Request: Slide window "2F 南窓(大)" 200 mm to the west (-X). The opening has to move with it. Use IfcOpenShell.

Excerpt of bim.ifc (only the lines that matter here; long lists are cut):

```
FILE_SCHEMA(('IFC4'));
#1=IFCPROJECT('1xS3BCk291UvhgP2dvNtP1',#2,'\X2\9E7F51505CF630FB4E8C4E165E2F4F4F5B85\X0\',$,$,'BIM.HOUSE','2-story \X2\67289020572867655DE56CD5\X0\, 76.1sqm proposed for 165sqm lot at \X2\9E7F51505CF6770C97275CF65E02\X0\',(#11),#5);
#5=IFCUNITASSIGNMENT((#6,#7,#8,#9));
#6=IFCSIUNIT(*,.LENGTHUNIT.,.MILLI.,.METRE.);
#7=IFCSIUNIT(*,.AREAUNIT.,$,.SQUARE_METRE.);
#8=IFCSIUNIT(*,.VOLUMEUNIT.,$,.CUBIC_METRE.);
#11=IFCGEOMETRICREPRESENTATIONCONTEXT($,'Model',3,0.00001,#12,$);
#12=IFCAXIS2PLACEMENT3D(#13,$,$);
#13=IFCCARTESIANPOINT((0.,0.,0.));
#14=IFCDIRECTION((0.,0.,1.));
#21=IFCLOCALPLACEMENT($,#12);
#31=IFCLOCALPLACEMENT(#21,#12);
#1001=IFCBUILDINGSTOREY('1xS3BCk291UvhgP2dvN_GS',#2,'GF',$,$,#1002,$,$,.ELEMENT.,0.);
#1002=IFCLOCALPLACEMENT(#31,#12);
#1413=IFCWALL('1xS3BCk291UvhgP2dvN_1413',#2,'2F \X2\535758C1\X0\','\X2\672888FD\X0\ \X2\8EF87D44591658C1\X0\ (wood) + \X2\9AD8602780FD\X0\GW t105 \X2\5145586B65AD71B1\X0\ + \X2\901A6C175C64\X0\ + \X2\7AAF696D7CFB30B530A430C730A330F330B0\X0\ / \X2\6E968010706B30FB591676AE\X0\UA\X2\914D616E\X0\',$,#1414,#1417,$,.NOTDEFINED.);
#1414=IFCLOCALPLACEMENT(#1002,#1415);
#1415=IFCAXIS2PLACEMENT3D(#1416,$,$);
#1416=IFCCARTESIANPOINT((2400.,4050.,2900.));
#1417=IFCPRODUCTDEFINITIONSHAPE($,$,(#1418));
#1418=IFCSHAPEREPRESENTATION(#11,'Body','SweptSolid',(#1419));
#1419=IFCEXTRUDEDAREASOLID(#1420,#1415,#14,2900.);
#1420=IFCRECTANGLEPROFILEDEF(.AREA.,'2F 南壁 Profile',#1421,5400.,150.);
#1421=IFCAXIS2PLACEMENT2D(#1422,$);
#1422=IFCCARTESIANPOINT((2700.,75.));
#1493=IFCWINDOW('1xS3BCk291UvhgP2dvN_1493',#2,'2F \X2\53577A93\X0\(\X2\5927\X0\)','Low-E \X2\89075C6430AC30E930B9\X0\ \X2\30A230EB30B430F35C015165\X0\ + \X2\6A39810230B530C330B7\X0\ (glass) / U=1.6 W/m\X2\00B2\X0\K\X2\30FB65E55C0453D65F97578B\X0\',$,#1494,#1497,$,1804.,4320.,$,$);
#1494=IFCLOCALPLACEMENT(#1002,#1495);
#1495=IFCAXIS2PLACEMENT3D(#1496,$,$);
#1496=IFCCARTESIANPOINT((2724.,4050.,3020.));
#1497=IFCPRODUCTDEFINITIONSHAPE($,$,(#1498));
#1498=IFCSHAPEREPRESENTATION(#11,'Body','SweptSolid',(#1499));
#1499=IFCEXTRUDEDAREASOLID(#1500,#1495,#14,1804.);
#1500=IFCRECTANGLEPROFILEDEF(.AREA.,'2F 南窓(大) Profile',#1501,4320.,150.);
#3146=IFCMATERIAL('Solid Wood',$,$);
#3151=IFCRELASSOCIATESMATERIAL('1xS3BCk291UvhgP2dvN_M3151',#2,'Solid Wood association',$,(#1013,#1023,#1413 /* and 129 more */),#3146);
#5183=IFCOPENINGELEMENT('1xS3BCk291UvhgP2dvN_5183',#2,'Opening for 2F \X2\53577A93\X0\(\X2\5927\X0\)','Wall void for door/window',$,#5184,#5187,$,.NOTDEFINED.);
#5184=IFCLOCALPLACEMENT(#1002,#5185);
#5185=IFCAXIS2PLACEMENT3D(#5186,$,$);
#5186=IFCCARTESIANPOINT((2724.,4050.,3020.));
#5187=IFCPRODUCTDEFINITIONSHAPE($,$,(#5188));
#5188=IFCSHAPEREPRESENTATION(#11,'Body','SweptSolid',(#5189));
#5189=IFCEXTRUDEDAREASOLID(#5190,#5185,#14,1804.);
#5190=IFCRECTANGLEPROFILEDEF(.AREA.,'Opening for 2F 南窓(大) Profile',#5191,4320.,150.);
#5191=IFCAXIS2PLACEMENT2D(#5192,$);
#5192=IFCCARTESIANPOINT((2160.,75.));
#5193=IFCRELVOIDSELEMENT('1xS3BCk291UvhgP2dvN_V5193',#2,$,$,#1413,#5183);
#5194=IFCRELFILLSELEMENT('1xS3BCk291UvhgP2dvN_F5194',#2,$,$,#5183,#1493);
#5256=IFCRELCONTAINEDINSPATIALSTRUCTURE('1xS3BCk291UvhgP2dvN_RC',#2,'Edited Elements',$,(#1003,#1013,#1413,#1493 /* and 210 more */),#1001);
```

```python
import ifcopenshell
import ifcopenshell.api.geometry
import ifcopenshell.util.placement
import ifcopenshell.util.unit

model = ifcopenshell.open("bim.ifc")
unit_scale = ifcopenshell.util.unit.calculate_unit_scale(model)

window = model.by_guid("1xS3BCk291UvhgP2dvN_1493")
opening = window.FillsVoids[0].RelatingOpeningElement
wall = opening.VoidsElements[0].RelatingBuildingElement

wall_matrix = ifcopenshell.util.placement.get_local_placement(wall.ObjectPlacement)
shift = wall_matrix[:3, 0] * -0.2 / unit_scale
before = ifcopenshell.util.placement.get_local_placement(window.ObjectPlacement)[:3, 3].copy()

# The window is not placed relative to its opening, so move both.
for product in (opening, window):
    matrix = ifcopenshell.util.placement.get_local_placement(product.ObjectPlacement)
    matrix[:3, 3] += shift
    ifcopenshell.api.geometry.edit_object_placement(model, product=product, matrix=matrix, is_si=False)

after = ifcopenshell.util.placement.get_local_placement(window.ObjectPlacement)[:3, 3]
print("window moved by", (after - before).round(3) + 0.0)

model.write("bim_edited.ifc")
```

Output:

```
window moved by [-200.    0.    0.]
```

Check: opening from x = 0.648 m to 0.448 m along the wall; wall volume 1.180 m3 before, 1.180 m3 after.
